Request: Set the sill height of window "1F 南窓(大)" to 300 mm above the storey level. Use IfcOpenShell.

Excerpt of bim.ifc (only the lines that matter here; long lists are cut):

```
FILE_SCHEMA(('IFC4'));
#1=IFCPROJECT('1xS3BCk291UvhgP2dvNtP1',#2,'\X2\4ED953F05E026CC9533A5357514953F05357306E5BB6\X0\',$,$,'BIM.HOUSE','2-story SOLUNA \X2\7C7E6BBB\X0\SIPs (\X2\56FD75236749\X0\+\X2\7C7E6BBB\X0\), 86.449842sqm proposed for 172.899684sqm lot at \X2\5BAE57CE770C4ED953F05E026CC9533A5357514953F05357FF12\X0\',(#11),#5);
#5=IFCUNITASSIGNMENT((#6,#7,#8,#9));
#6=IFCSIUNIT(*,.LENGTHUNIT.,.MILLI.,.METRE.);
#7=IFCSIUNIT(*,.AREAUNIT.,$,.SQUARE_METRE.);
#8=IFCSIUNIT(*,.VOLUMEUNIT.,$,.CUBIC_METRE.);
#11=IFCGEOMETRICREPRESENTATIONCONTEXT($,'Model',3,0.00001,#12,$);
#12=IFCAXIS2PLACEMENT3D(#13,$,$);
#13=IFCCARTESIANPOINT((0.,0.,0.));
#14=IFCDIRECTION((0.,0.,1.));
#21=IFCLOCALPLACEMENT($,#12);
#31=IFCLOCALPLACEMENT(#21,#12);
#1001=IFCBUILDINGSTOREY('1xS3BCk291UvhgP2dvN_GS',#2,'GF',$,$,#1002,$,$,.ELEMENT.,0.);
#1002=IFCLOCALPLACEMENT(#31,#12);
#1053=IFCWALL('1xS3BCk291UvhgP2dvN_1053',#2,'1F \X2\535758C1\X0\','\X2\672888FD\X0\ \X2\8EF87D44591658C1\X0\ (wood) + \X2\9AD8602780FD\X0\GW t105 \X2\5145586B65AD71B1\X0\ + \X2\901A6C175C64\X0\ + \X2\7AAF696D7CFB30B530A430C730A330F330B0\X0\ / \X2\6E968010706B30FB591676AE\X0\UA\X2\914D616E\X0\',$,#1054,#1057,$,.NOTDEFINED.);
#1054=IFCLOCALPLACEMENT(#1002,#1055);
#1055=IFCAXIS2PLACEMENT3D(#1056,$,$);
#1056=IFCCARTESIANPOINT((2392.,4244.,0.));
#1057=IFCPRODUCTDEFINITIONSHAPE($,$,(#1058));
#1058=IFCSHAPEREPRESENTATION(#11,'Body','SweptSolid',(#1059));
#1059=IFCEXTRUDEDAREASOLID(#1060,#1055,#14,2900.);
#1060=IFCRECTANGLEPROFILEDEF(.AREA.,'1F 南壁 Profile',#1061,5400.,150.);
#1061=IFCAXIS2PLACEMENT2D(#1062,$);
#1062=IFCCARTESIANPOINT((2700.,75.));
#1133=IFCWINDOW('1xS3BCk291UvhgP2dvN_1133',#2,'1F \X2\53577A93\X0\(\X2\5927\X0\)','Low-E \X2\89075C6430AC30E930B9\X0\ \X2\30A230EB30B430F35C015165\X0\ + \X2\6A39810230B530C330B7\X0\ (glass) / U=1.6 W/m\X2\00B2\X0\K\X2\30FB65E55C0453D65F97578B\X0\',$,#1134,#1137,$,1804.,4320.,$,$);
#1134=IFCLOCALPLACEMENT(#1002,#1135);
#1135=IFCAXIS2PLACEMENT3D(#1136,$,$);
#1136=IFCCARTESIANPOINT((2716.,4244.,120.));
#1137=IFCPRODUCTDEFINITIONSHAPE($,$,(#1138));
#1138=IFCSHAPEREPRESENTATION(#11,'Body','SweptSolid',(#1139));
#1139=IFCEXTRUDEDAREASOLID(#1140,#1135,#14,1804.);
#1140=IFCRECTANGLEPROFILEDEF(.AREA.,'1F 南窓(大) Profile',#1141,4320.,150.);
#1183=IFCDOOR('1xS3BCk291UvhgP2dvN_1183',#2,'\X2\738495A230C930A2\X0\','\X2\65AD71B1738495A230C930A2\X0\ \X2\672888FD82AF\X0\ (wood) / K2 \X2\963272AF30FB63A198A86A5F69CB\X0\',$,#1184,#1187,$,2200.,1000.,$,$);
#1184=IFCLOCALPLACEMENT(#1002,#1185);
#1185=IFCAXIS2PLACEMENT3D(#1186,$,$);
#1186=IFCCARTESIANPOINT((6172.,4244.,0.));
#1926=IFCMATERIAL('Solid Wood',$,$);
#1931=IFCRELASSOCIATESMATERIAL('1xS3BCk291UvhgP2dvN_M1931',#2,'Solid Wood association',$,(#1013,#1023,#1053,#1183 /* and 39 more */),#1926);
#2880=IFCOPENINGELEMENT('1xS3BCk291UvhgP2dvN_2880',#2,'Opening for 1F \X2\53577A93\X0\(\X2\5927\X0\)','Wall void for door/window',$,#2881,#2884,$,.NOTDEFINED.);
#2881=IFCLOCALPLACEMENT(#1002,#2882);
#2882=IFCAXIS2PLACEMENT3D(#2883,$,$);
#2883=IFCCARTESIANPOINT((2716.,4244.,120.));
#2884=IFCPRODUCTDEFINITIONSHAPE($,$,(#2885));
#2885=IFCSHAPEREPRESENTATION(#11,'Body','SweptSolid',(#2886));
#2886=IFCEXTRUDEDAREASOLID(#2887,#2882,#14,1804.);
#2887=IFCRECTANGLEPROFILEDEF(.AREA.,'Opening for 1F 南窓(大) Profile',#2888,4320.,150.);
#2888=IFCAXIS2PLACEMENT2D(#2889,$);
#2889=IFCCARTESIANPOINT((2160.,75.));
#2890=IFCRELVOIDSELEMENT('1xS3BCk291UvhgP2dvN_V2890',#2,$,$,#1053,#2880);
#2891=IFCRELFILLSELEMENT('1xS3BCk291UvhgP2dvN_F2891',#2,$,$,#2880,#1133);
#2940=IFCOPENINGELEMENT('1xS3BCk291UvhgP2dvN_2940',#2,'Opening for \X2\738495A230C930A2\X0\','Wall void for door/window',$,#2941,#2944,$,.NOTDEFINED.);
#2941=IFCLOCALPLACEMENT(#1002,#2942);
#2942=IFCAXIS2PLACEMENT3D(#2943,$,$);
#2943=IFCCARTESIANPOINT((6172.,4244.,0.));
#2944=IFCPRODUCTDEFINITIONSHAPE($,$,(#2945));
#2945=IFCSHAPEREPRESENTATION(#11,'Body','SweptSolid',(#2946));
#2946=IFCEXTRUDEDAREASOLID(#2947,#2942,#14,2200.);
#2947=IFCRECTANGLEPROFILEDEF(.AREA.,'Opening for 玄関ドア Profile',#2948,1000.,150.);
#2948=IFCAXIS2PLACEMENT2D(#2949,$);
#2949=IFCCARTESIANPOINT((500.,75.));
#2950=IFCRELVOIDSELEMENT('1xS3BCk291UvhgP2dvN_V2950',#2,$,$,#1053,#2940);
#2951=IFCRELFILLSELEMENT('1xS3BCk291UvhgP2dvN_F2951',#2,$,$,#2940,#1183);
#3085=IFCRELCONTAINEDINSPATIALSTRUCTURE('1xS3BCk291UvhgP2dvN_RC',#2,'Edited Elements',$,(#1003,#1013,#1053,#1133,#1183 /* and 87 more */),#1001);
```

```python
import numpy as np
import ifcopenshell
import ifcopenshell.api.geometry
import ifcopenshell.geom
import ifcopenshell.util.element
import ifcopenshell.util.placement
import ifcopenshell.util.shape
import ifcopenshell.util.unit

model = ifcopenshell.open("bim.ifc")
unit_scale = ifcopenshell.util.unit.calculate_unit_scale(model)

window = model.by_guid("1xS3BCk291UvhgP2dvN_1133")
opening = window.FillsVoids[0].RelatingOpeningElement
storey = ifcopenshell.util.element.get_container(window, ifc_class="IfcBuildingStorey")
level = ifcopenshell.util.placement.get_local_placement(storey.ObjectPlacement)[2, 3]

# The opening's origin need not be at the sill, so measure its lowest point.
shape = ifcopenshell.geom.create_shape(ifcopenshell.geom.settings(), opening)
bottom = ifcopenshell.util.shape.get_shape_bottom_elevation(shape, shape.geometry) / unit_scale
dz = level + 0.3 / unit_scale - bottom

shift = np.array([0.0, 0.0, dz])
# The window is not placed relative to its opening, so move both.
for product in (opening, window):
    matrix = ifcopenshell.util.placement.get_local_placement(product.ObjectPlacement)
    matrix[:3, 3] += shift
    ifcopenshell.api.geometry.edit_object_placement(model, product=product, matrix=matrix, is_si=False)

print(f"moved by {dz * unit_scale:+.3f} m")

model.write("bim_rev.ifc")
```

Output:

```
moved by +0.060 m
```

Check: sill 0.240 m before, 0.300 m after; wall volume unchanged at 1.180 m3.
